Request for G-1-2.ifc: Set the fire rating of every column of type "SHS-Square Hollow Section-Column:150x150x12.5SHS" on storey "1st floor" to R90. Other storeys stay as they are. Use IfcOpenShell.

First a look at what the model holds.

```python
import ifcopenshell
import ifcopenshell.util.element

model = ifcopenshell.open("G-1-2.ifc")
print(model.schema)
storey = next(s for s in model.by_type("IfcBuildingStorey") if s.Name == "1st floor")
columns = [e for e in ifcopenshell.util.element.get_decomposition(storey) if e.is_a("IfcColumn")]
seen = {}
for e in columns:
    element_type = ifcopenshell.util.element.get_type(e)
    key = (element_type.Name if element_type != e and element_type else None, ifcopenshell.util.element.get_pset(e, "Pset_ColumnCommon", "FireRating"))
    seen[key] = seen.get(key, 0) + 1
for (name, value), count in sorted(seen.items(), key=str):
    print(count, "x", name, "|", value)
```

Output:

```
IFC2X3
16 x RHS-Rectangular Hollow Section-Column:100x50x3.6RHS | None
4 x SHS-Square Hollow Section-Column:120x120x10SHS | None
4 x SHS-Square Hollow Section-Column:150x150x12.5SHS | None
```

```python
import ifcopenshell
import ifcopenshell.api.pset
import ifcopenshell.util.element

model = ifcopenshell.open("G-1-2.ifc")

storey = next(s for s in model.by_type("IfcBuildingStorey") if s.Name == "1st floor")
columns = [e for e in ifcopenshell.util.element.get_decomposition(storey) if e.is_a("IfcColumn")]

count = 0
for e in columns:
    element_type = ifcopenshell.util.element.get_type(e)
    if element_type in (None, e) or element_type.Name != "SHS-Square Hollow Section-Column:150x150x12.5SHS":
        continue
    # add_pset returns the element's existing set when there is one.
    pset = ifcopenshell.api.pset.add_pset(model, product=e, name="Pset_ColumnCommon")
    ifcopenshell.api.pset.edit_pset(model, pset=pset, properties={"FireRating": "R90"})
    count += 1

print(count, "columns updated")

model.write("G-1-2_updated.ifc")
```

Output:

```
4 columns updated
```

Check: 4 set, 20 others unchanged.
